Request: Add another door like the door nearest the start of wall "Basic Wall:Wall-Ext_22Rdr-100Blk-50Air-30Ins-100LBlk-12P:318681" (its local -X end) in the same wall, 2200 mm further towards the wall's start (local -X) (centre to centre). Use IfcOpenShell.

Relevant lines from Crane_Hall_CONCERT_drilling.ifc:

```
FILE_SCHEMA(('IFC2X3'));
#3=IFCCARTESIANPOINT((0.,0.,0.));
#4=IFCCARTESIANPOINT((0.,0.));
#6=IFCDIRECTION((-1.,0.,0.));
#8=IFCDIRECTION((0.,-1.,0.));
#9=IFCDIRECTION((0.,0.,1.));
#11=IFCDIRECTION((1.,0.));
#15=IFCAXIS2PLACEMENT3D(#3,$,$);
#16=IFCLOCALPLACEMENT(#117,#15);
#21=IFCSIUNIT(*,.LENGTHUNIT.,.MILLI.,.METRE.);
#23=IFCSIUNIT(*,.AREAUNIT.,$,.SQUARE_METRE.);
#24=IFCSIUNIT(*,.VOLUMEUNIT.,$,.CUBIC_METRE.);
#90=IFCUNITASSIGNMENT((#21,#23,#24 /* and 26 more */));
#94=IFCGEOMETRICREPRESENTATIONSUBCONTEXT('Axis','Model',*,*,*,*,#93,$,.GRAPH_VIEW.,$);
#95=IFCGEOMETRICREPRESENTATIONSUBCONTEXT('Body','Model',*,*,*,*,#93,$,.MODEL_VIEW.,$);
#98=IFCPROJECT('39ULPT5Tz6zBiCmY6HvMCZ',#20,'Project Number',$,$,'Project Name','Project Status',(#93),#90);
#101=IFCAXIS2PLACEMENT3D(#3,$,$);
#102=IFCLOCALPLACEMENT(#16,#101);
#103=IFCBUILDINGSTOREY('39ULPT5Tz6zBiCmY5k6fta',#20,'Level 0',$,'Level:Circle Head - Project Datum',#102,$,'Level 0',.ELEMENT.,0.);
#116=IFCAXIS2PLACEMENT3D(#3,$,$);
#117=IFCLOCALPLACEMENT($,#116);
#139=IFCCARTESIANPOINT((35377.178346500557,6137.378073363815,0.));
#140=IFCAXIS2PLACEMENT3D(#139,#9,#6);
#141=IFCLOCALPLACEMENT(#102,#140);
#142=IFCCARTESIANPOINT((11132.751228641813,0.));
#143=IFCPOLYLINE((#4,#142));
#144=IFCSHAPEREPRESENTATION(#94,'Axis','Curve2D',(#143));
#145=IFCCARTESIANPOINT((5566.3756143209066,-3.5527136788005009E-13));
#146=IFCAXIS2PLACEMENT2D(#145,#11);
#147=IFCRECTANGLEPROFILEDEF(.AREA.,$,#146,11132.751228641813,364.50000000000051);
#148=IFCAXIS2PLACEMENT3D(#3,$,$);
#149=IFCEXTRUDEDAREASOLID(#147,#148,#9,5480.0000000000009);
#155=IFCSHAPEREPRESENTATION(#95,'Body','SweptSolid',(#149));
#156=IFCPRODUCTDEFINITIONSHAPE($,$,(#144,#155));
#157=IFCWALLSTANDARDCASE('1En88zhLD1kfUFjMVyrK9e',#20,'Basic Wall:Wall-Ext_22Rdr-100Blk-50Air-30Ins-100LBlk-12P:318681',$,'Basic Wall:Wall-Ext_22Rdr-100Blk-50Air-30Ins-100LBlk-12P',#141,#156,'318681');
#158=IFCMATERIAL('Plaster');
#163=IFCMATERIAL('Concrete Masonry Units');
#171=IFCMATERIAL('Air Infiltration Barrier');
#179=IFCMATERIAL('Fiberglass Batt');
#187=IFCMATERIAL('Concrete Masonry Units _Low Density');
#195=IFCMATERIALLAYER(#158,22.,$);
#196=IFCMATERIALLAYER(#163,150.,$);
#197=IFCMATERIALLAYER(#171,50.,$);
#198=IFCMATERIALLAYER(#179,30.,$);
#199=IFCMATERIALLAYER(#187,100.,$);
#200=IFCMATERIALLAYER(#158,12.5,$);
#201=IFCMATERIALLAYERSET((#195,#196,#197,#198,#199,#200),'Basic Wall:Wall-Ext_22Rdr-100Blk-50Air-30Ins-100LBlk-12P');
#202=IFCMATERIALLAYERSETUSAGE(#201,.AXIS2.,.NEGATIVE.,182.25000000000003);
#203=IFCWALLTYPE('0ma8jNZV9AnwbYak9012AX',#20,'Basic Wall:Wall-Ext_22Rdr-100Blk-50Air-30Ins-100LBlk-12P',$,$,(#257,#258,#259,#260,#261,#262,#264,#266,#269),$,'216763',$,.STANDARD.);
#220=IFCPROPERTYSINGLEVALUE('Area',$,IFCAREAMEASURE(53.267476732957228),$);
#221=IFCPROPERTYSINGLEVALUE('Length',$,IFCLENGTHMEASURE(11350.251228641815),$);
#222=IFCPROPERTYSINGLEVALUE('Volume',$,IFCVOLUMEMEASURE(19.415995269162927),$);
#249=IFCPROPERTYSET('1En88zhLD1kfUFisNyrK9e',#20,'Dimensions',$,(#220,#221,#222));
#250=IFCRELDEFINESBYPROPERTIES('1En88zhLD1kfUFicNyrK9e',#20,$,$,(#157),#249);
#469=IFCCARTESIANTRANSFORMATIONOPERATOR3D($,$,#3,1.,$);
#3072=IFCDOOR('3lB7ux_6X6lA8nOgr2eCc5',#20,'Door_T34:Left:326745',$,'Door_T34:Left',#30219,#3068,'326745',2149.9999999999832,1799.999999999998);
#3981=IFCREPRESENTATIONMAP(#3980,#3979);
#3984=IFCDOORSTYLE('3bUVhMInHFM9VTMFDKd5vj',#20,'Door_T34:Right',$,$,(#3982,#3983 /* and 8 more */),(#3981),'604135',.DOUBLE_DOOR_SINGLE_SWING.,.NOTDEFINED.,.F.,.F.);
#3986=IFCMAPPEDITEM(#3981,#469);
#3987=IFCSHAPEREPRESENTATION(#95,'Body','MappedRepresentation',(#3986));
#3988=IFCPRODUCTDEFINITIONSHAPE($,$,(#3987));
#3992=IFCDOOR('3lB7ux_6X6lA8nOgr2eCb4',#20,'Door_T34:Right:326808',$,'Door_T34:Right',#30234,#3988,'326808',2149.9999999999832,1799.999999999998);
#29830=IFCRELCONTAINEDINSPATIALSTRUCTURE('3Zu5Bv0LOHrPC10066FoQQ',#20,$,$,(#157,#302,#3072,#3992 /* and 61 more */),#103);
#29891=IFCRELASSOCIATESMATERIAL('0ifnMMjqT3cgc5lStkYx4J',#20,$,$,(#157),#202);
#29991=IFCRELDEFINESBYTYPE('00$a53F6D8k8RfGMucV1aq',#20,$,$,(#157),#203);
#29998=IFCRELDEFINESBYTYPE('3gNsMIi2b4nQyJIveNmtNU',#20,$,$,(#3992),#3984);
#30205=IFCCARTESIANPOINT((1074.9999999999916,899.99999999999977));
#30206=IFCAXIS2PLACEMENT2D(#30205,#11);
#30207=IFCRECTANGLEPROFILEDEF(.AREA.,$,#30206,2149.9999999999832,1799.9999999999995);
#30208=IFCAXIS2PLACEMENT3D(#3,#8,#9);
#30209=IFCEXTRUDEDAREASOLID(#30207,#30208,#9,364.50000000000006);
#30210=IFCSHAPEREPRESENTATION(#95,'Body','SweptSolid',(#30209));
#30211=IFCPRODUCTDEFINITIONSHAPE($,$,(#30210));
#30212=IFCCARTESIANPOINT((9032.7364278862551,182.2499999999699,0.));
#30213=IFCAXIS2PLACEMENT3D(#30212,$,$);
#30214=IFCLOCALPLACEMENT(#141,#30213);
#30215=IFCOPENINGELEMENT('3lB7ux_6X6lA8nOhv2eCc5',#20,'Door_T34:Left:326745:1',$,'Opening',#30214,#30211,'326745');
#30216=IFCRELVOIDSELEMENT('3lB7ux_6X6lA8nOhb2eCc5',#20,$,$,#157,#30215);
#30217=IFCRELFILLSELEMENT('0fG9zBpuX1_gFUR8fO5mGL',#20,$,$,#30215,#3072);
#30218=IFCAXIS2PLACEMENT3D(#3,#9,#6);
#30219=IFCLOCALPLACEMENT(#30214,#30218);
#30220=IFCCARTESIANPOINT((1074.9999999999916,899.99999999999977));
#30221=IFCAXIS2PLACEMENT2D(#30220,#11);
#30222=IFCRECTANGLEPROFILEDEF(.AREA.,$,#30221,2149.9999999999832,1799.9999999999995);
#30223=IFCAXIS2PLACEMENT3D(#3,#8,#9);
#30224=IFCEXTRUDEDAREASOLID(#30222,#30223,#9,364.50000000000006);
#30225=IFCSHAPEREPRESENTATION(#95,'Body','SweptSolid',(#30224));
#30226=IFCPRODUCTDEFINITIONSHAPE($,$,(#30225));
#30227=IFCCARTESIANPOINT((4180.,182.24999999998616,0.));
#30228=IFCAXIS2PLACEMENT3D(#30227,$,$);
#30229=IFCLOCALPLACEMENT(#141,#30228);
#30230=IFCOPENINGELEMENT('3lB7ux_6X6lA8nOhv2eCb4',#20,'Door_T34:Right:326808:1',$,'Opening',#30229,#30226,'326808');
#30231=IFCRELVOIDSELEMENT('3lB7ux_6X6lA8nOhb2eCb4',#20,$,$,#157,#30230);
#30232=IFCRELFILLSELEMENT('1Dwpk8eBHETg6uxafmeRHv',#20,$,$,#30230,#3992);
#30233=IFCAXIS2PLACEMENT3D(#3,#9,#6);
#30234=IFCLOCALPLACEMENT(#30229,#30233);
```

```python
import ifcopenshell
import ifcopenshell.api.feature
import ifcopenshell.api.geometry
import ifcopenshell.api.pset
import ifcopenshell.api.root
import ifcopenshell.geom
import ifcopenshell.util.element
import ifcopenshell.util.placement
import ifcopenshell.util.shape
import ifcopenshell.util.unit

model = ifcopenshell.open("Crane_Hall_CONCERT_drilling.ifc")
unit_scale = ifcopenshell.util.unit.calculate_unit_scale(model)
area_scale = ifcopenshell.util.unit.calculate_unit_scale(model, "AREAUNIT")
volume_scale = ifcopenshell.util.unit.calculate_unit_scale(model, "VOLUMEUNIT")
settings = ifcopenshell.geom.settings()


def volume(element):
    """Net volume in cubic metres, openings subtracted."""
    shape = ifcopenshell.geom.create_shape(settings, element)
    return ifcopenshell.util.shape.get_volume(shape.geometry)


def reuse_history(source, copy):
    """copy_class also copies each property set's owner history, people and application; keep the originals."""
    for rel in copy.IsDefinedBy:
        if rel.is_a("IfcRelDefinesByProperties") and (history := rel.RelatingPropertyDefinition.OwnerHistory):
            rel.RelatingPropertyDefinition.OwnerHistory = source.OwnerHistory
            ifcopenshell.util.element.remove_deep2(model, history)


door = model.by_id(3992)
opening = door.FillsVoids[0].RelatingOpeningElement
wall = opening.VoidsElements[0].RelatingBuildingElement
before = volume(wall)
shift = ifcopenshell.util.placement.get_local_placement(wall.ObjectPlacement)[:3, 0] * -2.2 / unit_scale

# copy_class copies the void relationship, type, container and properties, but no geometry.
new_opening = ifcopenshell.api.root.copy_class(model, product=opening)
new_opening.Representation = ifcopenshell.util.element.copy_deep(
    model, opening.Representation, exclude=["IfcGeometricRepresentationContext", "IfcRepresentationMap"]
)
new_opening.Name = "Door_T34:Right"
new_opening.Tag = None
new_door = ifcopenshell.api.root.copy_class(model, product=door)
new_door.Representation = ifcopenshell.util.element.copy_deep(
    model, door.Representation, exclude=["IfcGeometricRepresentationContext", "IfcRepresentationMap"]
)
new_door.Name = "Door_T34:Right"
new_door.Tag = None
reuse_history(door, new_door)
fills = ifcopenshell.api.feature.add_filling(model, opening=new_opening, element=new_door)
fills.OwnerHistory = new_door.OwnerHistory  # required in IFC2X3

for old, new in ((opening, new_opening), (door, new_door)):
    matrix = ifcopenshell.util.placement.get_local_placement(old.ObjectPlacement)
    matrix[:3, 3] += shift
    ifcopenshell.api.geometry.edit_object_placement(model, product=new, matrix=matrix, is_si=False)

after = volume(wall)
thickness = 0.3645  # wall thickness in metres

# Update the wall's stored quantities.
pset = model.by_id(ifcopenshell.util.element.get_pset(wall, "Dimensions", should_inherit=False)["id"])
ifcopenshell.api.pset.edit_pset(model, pset=pset, properties={
    "Area": model.create_entity("IfcAreaMeasure", after / thickness / area_scale),
    "Volume": model.create_entity("IfcVolumeMeasure", after / volume_scale),
})

print(f"wall volume {before:.3f} -> {after:.3f} m3")

model.write("Crane_Hall_CONCERT_drilling_updated.ifc")
```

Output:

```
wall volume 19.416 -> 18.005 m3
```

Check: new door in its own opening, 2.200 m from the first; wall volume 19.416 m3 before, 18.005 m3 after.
